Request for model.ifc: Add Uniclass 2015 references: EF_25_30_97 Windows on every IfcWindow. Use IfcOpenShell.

First a look at what the model holds.

```python
import ifcopenshell

model = ifcopenshell.open("model.ifc")
print(model.schema)
print("classifications:", [c.Name for c in model.by_type("IfcClassification")])
for ifc_class in ("IfcDoor", "IfcRoof", "IfcStair", "IfcWall", "IfcWindow"):
    print(ifc_class, len(model.by_type(ifc_class)))
```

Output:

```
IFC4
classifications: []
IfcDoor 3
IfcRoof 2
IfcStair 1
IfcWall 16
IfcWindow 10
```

```python
import ifcopenshell
import ifcopenshell.api.classification

model = ifcopenshell.open("model.ifc")

system = ifcopenshell.api.classification.add_classification(model, classification="Uniclass 2015")

codes = {
    "IfcWindow": ("EF_25_30_97", "Windows"),
}
for ifc_class, (code, name) in codes.items():
    products = model.by_type(ifc_class)
    ifcopenshell.api.classification.add_reference(
        model, products=products, classification=system, identification=code, name=name
    )
    print(code, len(products))

model.write("model_rev.ifc")
```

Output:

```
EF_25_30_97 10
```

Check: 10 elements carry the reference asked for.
